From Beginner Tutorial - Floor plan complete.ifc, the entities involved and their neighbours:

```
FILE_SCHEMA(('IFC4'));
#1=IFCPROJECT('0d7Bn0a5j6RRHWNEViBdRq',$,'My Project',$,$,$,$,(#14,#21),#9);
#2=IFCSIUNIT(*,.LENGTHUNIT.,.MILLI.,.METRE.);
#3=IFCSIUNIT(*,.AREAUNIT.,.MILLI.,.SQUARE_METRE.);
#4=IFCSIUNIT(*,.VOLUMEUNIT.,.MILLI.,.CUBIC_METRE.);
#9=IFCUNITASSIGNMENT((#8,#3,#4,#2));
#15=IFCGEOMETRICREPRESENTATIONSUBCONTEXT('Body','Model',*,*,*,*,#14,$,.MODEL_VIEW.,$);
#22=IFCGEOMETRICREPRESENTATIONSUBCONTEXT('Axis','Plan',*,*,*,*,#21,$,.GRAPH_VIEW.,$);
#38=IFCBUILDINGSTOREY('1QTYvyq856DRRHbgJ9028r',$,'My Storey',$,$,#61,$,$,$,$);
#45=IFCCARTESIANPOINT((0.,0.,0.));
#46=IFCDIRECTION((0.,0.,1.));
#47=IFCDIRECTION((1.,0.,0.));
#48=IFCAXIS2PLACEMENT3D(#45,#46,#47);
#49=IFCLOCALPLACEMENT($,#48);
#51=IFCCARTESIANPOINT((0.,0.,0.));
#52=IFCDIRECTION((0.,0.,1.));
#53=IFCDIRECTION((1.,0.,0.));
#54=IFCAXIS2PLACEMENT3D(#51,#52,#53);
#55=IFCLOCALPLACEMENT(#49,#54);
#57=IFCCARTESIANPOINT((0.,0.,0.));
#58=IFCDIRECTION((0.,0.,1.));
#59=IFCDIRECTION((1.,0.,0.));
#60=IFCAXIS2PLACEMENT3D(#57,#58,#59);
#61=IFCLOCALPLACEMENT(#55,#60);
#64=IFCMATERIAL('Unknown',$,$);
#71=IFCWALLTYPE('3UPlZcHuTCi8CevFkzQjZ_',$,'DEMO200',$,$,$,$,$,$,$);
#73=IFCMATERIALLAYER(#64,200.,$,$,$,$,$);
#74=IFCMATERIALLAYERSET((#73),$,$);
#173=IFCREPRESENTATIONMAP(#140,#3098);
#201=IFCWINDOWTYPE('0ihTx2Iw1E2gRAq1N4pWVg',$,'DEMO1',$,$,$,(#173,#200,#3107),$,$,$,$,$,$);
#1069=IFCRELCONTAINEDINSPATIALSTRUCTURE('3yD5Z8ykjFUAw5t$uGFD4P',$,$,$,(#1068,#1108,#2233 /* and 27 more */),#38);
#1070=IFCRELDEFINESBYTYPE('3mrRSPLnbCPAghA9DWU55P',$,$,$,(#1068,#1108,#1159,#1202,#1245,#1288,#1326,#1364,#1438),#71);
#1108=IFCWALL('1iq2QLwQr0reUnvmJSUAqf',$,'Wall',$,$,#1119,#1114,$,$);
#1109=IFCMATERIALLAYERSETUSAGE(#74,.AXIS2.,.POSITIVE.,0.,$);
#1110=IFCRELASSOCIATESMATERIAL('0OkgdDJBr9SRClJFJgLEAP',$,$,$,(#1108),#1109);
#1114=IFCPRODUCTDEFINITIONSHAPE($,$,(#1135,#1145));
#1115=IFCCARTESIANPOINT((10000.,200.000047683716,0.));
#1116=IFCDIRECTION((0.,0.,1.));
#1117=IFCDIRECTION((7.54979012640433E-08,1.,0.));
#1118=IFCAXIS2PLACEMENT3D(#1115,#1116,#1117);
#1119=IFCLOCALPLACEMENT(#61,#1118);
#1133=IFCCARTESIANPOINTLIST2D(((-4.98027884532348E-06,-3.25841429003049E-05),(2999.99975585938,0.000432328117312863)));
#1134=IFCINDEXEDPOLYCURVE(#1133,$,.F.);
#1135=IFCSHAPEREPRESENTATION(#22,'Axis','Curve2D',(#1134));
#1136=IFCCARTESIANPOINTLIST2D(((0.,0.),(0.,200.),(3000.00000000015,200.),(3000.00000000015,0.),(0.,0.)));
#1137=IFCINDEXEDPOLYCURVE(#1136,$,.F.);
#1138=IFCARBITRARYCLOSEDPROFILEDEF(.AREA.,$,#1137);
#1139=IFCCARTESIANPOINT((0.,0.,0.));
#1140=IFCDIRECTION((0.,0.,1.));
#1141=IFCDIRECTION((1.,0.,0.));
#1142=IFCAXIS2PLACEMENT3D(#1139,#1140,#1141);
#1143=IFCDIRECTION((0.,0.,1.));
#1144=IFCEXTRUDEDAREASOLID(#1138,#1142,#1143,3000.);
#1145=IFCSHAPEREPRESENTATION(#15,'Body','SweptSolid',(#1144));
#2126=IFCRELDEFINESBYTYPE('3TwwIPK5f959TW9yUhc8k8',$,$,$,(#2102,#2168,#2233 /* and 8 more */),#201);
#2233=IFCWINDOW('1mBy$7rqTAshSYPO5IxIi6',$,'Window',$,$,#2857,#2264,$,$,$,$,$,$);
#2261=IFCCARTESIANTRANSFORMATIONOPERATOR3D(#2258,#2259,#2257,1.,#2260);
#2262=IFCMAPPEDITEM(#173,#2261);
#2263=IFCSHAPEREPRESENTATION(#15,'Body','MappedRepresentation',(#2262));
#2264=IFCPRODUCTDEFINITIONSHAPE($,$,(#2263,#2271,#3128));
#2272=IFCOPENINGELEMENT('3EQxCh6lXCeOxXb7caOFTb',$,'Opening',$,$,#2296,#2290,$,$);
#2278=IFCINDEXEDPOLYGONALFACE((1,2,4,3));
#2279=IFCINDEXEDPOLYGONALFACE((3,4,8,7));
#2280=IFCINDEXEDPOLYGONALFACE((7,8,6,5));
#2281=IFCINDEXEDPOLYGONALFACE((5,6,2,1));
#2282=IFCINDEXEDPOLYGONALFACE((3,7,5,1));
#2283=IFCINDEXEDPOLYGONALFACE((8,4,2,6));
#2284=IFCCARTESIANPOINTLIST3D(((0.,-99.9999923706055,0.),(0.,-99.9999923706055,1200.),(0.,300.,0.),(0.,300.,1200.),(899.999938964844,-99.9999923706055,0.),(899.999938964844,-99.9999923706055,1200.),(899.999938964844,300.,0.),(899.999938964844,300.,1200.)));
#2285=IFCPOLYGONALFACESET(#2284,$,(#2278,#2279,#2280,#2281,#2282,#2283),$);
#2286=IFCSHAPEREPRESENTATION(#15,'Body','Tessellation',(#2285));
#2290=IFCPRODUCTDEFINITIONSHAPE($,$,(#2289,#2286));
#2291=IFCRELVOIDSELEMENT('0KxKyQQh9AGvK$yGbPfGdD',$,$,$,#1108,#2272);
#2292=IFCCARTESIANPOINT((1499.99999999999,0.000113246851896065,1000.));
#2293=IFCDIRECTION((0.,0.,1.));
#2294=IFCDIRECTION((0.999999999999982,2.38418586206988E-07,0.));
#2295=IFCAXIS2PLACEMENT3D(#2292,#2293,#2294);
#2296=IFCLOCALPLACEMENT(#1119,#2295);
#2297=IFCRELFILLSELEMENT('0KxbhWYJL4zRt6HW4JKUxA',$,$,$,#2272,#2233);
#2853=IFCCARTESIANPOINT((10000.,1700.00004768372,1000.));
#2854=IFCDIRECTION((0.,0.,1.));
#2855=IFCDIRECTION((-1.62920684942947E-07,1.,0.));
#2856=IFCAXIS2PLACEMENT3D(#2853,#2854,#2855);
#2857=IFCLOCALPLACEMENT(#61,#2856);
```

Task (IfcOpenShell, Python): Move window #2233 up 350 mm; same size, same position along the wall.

```python
import numpy as np
import ifcopenshell
import ifcopenshell.api.geometry
import ifcopenshell.util.placement
import ifcopenshell.util.unit

model = ifcopenshell.open("Beginner Tutorial - Floor plan complete.ifc")
unit_scale = ifcopenshell.util.unit.calculate_unit_scale(model)

window = model.by_id(2233)
opening = window.FillsVoids[0].RelatingOpeningElement
dz = 0.35 / unit_scale

shift = np.array([0.0, 0.0, dz])
# The window is not placed relative to its opening, so move both.
for product in (opening, window):
    matrix = ifcopenshell.util.placement.get_local_placement(product.ObjectPlacement)
    matrix[:3, 3] += shift
    ifcopenshell.api.geometry.edit_object_placement(model, product=product, matrix=matrix, is_si=False)

print(f"moved by {dz * unit_scale:+.3f} m")

model.write("Beginner Tutorial - Floor plan complete_edited.ifc")
```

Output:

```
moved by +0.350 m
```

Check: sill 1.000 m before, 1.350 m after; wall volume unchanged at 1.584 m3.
